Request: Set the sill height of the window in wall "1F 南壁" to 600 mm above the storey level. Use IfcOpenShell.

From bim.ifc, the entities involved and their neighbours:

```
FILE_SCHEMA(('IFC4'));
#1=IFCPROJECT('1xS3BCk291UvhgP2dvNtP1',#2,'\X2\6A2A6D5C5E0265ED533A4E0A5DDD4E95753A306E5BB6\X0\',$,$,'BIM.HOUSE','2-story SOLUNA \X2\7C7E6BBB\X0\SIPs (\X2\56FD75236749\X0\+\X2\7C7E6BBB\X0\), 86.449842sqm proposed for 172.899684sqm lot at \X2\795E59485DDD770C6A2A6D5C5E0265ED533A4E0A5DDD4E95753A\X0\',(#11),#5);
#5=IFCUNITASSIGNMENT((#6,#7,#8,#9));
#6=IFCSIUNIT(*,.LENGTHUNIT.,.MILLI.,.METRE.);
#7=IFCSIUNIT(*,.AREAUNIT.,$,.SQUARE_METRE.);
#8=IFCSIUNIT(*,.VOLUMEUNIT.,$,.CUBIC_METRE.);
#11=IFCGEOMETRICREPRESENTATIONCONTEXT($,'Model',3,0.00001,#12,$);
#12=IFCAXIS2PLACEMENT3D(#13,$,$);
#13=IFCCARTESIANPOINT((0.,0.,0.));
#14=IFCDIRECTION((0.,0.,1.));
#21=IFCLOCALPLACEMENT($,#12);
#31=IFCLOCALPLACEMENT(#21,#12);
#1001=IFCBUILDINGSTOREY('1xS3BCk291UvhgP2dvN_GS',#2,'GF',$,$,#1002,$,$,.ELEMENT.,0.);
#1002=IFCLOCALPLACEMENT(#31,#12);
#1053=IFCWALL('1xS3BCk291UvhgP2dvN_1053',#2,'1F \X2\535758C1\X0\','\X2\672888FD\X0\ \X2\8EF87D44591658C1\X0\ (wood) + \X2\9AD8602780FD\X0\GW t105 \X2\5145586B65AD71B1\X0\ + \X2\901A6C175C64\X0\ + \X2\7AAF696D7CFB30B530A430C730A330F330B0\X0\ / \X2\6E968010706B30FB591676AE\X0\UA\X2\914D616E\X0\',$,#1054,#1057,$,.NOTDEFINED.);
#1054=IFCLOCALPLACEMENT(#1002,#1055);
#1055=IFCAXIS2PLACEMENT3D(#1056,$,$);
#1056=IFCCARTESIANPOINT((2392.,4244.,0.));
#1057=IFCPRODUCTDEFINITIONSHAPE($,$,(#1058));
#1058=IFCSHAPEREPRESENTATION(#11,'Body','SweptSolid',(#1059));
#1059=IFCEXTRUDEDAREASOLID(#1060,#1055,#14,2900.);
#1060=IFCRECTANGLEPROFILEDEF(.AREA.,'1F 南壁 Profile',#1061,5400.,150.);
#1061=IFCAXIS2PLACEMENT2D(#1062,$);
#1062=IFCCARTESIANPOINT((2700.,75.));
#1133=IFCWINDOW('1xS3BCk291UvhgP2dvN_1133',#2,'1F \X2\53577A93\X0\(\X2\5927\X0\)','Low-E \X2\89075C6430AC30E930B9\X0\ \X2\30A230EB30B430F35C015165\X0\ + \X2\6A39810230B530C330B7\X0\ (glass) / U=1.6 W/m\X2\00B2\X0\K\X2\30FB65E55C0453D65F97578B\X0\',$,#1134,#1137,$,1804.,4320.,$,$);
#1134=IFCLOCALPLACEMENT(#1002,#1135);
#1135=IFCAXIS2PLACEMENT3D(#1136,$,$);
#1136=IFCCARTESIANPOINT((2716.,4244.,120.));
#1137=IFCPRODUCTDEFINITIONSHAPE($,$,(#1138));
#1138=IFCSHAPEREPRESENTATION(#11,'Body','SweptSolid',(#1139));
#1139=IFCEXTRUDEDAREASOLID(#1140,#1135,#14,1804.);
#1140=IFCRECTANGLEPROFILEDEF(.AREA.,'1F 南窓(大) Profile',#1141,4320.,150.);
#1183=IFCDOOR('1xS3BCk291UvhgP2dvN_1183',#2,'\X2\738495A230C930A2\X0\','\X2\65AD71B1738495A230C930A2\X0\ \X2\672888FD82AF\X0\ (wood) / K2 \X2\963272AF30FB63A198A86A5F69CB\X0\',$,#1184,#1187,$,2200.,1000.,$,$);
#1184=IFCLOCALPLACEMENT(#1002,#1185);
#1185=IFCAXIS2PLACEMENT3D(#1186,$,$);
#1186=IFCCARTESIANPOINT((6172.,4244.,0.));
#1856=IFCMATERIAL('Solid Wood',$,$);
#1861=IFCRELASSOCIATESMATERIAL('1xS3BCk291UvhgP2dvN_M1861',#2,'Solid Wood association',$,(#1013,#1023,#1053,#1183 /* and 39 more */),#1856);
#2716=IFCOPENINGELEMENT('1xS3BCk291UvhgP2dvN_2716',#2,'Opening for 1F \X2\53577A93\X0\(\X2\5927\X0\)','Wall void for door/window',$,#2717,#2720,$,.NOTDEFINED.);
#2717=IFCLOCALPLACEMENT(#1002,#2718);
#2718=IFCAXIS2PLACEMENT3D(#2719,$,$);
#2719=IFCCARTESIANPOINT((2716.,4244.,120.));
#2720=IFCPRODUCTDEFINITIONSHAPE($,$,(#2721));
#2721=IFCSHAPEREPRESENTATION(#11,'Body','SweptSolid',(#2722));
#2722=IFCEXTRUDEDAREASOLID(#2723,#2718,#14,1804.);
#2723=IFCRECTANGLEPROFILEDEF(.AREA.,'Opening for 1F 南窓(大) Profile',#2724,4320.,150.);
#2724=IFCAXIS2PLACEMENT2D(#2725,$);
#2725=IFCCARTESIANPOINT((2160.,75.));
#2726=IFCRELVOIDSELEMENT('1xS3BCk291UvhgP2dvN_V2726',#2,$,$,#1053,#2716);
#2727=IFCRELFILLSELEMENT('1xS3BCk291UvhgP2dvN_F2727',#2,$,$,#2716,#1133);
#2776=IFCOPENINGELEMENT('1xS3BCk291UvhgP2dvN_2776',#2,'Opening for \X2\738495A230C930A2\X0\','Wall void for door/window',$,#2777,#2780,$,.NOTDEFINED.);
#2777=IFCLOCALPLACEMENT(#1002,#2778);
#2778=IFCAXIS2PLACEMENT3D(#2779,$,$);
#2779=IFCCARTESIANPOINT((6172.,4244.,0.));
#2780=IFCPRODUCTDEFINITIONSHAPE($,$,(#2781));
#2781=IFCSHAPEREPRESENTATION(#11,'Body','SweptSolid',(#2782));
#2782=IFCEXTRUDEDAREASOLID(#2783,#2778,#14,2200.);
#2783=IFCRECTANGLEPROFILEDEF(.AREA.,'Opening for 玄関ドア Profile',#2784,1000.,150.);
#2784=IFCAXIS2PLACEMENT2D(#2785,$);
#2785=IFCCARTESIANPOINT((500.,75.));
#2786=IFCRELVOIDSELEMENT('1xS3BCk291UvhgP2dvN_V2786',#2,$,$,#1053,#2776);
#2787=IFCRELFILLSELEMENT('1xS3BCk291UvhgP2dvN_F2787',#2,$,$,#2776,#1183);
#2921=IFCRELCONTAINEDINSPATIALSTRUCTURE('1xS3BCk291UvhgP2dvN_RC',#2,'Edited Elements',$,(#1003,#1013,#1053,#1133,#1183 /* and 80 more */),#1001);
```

```python
import numpy as np
import ifcopenshell
import ifcopenshell.api.geometry
import ifcopenshell.geom
import ifcopenshell.util.element
import ifcopenshell.util.placement
import ifcopenshell.util.shape
import ifcopenshell.util.unit

model = ifcopenshell.open("bim.ifc")
unit_scale = ifcopenshell.util.unit.calculate_unit_scale(model)

window = model.by_id(1133)
opening = window.FillsVoids[0].RelatingOpeningElement
storey = ifcopenshell.util.element.get_container(window, ifc_class="IfcBuildingStorey")
level = ifcopenshell.util.placement.get_local_placement(storey.ObjectPlacement)[2, 3]

# The opening's origin need not be at the sill, so measure its lowest point.
shape = ifcopenshell.geom.create_shape(ifcopenshell.geom.settings(), opening)
bottom = ifcopenshell.util.shape.get_shape_bottom_elevation(shape, shape.geometry) / unit_scale
dz = level + 600.0 - bottom

shift = np.array([0.0, 0.0, dz])
# The window is not placed relative to its opening, so move both.
for product in (opening, window):
    matrix = ifcopenshell.util.placement.get_local_placement(product.ObjectPlacement)
    matrix[:3, 3] += shift
    ifcopenshell.api.geometry.edit_object_placement(model, product=product, matrix=matrix, is_si=False)

print(f"moved by {dz * unit_scale:+.3f} m")

model.write("bim_rev.ifc")
```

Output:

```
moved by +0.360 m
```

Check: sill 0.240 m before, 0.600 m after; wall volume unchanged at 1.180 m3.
